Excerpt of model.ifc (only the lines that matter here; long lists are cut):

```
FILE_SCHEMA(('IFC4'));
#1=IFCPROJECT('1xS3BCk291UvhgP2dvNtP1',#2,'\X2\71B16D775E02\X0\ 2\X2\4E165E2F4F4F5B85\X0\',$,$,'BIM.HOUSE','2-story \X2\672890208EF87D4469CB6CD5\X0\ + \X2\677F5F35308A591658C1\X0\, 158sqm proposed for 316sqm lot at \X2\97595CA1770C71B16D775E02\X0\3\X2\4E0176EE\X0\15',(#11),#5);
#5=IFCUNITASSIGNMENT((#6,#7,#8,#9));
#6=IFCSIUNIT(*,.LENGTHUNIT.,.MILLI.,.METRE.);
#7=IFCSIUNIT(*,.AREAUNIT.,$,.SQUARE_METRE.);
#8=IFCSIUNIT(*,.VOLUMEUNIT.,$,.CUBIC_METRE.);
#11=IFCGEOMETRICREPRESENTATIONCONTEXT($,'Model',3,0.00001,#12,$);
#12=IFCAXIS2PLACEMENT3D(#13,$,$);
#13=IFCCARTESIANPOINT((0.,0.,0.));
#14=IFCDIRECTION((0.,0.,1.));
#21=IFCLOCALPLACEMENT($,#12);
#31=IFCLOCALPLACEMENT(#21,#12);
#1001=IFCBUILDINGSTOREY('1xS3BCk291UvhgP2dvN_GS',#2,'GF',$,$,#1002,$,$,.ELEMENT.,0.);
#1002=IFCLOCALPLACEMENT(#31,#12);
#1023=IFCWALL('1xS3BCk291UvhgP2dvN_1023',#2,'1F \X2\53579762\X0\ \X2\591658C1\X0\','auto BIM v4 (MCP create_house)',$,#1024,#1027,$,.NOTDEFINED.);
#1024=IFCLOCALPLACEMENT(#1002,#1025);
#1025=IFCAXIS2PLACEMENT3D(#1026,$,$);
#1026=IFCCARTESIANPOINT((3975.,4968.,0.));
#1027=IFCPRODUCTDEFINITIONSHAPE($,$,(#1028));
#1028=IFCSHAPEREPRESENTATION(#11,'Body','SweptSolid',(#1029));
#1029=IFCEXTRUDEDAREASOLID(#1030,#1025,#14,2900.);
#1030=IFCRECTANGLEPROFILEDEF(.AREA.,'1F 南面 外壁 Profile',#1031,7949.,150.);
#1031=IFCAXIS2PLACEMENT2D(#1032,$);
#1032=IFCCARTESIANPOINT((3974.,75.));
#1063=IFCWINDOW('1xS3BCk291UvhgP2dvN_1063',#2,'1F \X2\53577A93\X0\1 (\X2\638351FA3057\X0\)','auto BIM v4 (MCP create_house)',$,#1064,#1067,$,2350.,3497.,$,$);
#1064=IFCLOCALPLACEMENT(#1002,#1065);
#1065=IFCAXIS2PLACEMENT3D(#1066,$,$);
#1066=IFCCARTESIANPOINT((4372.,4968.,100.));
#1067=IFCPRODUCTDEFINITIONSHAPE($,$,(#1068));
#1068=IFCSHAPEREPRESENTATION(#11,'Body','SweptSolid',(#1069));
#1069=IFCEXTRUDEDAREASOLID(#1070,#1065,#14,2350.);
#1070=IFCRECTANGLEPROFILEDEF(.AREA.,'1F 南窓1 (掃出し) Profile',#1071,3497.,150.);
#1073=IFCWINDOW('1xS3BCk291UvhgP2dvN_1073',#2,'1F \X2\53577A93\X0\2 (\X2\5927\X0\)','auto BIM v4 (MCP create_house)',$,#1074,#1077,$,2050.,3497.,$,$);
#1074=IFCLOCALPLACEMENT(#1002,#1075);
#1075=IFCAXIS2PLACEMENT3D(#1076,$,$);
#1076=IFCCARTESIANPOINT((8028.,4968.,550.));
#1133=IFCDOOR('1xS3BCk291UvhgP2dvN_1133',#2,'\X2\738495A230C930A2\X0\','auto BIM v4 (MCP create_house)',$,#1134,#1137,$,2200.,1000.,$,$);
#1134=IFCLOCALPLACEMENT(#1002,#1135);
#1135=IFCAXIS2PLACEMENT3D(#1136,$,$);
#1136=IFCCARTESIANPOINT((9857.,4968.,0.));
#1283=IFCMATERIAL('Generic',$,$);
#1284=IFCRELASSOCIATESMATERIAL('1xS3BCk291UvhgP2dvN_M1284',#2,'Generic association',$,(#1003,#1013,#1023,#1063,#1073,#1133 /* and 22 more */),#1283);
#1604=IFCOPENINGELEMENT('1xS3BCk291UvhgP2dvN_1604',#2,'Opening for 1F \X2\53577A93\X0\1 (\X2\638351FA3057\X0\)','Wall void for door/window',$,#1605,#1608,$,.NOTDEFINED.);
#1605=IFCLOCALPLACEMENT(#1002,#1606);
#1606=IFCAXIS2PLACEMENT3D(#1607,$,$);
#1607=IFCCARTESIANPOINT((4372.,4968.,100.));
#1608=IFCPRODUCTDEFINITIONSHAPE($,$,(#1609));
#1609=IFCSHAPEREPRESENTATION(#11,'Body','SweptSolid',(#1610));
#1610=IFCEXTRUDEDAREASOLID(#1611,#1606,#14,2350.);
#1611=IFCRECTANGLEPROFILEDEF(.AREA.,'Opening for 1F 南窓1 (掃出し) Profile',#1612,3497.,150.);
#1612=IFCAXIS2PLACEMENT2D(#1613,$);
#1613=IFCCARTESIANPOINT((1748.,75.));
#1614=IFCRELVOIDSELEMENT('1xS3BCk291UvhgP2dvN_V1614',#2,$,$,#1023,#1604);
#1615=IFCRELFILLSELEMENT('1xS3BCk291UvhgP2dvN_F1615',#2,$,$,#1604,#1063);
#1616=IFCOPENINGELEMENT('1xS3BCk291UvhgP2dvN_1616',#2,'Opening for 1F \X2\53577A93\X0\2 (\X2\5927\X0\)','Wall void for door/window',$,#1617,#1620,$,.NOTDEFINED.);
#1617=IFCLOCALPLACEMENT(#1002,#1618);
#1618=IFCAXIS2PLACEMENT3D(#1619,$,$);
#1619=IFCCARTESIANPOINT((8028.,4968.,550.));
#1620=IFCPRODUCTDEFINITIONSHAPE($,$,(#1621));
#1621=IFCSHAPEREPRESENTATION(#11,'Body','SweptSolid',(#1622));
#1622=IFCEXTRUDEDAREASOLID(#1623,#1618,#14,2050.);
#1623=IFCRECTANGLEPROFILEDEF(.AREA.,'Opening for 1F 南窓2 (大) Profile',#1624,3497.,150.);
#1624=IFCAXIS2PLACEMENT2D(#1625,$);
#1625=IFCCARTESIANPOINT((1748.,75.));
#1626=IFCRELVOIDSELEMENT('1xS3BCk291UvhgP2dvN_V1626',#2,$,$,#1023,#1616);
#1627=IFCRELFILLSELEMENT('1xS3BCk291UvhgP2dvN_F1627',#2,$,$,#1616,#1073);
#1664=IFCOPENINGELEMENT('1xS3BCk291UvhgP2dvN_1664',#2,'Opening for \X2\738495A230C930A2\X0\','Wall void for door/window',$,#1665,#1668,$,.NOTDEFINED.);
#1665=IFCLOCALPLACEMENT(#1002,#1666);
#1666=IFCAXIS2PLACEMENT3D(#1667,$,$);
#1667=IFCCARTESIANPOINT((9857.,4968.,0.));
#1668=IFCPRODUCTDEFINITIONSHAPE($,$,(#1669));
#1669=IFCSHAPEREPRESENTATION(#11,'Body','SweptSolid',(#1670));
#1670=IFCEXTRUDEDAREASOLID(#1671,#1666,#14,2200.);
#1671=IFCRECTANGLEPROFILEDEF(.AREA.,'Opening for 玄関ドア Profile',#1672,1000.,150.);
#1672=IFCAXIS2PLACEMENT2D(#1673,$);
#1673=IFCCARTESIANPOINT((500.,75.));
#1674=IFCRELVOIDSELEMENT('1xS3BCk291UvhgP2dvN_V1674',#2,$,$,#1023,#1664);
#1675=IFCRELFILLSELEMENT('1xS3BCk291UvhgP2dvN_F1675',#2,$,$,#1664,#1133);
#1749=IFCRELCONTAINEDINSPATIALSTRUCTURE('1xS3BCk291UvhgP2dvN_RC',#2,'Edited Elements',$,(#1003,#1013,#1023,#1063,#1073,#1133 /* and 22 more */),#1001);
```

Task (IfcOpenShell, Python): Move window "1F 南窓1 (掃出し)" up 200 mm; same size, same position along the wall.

```python
import numpy as np
import ifcopenshell
import ifcopenshell.api.geometry
import ifcopenshell.util.placement
import ifcopenshell.util.unit

model = ifcopenshell.open("model.ifc")
unit_scale = ifcopenshell.util.unit.calculate_unit_scale(model)

window = model.by_guid("1xS3BCk291UvhgP2dvN_1063")
opening = window.FillsVoids[0].RelatingOpeningElement
dz = 200.0

shift = np.array([0.0, 0.0, dz])
# The window is not placed relative to its opening, so move both.
for product in (opening, window):
    matrix = ifcopenshell.util.placement.get_local_placement(product.ObjectPlacement)
    matrix[:3, 3] += shift
    ifcopenshell.api.geometry.edit_object_placement(model, product=product, matrix=matrix, is_si=False)

print(f"moved by {dz * unit_scale:+.3f} m")

model.write("model_updated.ifc")
```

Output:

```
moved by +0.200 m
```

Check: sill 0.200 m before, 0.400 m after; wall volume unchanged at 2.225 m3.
